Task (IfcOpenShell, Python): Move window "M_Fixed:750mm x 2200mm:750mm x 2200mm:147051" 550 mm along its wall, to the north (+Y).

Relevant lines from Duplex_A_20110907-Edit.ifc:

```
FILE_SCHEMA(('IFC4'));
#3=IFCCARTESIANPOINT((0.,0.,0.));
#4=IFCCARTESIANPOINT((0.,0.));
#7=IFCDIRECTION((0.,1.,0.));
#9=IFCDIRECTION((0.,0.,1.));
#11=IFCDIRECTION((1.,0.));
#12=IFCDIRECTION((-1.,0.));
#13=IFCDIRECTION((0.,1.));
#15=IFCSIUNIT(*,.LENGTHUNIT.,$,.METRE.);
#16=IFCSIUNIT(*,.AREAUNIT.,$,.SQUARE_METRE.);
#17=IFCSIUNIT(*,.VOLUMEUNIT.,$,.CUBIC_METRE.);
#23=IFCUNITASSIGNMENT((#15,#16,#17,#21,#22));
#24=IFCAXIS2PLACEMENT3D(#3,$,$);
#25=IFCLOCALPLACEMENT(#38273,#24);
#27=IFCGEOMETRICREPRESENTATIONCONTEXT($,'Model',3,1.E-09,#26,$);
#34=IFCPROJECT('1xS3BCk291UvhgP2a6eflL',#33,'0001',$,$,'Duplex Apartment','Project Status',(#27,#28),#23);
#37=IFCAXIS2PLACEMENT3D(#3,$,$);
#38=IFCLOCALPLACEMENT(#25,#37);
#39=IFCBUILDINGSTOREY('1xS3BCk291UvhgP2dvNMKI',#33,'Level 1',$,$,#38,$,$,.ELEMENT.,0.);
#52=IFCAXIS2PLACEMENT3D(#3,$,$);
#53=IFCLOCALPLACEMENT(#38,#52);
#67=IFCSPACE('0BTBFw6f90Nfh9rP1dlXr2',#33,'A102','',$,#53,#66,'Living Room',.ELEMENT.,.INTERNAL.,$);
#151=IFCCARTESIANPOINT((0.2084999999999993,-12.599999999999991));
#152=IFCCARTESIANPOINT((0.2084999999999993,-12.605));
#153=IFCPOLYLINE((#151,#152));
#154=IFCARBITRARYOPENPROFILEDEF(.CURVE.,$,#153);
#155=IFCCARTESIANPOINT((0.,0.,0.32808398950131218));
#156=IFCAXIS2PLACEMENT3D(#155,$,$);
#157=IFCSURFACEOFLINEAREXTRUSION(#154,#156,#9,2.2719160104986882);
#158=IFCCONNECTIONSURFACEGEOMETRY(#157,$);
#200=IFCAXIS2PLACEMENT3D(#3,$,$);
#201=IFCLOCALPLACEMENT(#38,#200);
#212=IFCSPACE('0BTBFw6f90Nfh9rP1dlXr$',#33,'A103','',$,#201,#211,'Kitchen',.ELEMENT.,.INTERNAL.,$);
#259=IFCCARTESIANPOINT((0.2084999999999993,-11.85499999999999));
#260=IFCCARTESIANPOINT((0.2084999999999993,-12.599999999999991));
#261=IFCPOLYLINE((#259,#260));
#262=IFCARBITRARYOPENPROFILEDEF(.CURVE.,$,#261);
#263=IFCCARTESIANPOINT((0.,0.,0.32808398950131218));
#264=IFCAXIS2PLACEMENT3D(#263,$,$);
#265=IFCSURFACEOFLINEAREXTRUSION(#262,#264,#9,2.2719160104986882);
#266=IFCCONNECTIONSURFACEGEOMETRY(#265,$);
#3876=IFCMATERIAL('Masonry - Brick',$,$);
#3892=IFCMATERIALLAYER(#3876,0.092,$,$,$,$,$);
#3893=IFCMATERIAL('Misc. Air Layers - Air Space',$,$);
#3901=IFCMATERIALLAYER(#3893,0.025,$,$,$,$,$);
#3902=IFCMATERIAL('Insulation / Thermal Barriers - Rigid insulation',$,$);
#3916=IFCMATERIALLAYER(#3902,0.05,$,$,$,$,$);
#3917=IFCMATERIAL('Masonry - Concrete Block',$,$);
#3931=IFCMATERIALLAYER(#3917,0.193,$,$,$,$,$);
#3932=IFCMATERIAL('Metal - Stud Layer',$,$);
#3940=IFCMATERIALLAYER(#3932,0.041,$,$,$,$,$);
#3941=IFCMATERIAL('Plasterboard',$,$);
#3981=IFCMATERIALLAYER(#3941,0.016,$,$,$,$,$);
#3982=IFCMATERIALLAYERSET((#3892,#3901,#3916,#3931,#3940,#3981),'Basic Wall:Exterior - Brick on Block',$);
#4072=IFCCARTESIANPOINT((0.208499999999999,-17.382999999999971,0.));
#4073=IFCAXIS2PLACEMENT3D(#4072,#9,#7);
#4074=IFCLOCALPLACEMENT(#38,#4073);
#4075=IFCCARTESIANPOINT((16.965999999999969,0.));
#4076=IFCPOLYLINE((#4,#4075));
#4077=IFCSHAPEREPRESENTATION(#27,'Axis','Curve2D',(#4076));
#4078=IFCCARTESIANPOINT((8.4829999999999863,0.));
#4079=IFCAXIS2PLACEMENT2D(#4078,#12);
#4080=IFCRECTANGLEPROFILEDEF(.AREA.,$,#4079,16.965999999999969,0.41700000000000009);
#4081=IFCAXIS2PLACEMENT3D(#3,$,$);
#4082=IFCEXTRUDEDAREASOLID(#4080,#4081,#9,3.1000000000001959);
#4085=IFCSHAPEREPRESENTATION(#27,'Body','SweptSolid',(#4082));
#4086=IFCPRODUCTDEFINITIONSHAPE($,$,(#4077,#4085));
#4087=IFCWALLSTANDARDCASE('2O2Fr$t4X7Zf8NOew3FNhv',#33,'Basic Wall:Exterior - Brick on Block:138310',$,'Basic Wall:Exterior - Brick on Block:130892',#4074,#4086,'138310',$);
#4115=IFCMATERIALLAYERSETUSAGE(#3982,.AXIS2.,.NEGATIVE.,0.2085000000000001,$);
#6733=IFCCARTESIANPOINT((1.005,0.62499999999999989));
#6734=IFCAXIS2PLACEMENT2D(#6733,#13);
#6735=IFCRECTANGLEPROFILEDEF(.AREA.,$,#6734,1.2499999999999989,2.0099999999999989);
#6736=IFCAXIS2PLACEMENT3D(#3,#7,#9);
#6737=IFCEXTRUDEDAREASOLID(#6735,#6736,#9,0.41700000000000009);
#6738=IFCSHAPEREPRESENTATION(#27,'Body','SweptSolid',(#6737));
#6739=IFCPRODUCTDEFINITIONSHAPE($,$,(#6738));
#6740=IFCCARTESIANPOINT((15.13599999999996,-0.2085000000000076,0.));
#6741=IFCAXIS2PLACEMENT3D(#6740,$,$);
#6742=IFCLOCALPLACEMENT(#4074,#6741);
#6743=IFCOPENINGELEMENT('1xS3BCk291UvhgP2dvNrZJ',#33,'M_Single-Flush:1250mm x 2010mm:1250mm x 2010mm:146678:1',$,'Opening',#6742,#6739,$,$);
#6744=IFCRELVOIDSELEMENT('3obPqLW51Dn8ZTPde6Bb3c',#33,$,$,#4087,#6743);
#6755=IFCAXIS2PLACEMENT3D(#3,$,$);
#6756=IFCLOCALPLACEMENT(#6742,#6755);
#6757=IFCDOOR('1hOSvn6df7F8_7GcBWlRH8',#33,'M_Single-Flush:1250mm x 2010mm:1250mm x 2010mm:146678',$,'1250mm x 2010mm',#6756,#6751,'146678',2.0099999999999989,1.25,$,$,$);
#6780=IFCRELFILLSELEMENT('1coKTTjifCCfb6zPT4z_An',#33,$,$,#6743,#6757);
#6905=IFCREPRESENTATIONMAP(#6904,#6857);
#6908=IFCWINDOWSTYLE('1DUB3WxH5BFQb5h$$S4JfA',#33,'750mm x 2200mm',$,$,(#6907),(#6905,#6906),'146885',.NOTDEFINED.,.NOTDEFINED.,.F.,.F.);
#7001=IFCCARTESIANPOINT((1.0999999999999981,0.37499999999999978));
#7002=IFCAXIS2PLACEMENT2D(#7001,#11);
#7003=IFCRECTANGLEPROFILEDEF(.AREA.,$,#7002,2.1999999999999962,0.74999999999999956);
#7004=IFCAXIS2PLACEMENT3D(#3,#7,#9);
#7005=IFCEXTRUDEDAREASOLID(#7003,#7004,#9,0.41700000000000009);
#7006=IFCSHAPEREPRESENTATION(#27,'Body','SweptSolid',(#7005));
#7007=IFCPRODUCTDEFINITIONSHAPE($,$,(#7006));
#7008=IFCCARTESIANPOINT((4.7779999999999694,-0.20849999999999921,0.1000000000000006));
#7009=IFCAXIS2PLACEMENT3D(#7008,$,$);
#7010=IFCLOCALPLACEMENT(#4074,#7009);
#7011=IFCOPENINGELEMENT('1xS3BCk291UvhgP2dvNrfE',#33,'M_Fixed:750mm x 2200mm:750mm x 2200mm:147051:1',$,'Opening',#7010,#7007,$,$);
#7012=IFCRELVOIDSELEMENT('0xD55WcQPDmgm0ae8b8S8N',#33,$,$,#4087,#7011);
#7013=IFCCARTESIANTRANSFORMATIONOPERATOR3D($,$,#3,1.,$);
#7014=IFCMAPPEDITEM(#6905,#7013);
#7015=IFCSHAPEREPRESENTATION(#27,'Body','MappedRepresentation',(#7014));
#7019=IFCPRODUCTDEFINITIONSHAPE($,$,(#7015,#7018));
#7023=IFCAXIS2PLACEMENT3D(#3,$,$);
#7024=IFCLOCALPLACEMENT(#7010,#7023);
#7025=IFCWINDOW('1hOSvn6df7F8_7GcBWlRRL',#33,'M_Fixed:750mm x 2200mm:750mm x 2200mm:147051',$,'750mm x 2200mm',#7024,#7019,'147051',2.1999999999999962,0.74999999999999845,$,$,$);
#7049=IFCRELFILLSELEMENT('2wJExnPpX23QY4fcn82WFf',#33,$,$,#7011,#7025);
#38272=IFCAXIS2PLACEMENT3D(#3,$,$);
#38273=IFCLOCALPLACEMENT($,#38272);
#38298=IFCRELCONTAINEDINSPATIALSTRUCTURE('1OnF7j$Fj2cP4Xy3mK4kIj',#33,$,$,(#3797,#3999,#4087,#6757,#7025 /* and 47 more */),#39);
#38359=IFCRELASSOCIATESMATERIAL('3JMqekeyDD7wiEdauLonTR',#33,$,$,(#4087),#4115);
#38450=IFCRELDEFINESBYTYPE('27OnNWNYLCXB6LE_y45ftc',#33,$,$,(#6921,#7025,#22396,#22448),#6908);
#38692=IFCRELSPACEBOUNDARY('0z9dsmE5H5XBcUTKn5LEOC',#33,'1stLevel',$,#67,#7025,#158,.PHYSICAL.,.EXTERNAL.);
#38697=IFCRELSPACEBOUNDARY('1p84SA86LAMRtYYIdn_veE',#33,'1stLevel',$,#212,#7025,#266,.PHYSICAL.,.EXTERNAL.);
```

```python
import numpy as np
import ifcopenshell
import ifcopenshell.api.geometry
import ifcopenshell.util.placement
import ifcopenshell.util.unit

model = ifcopenshell.open("Duplex_A_20110907-Edit.ifc")
unit_scale = ifcopenshell.util.unit.calculate_unit_scale(model)

window = model.by_guid("1hOSvn6df7F8_7GcBWlRRL")
opening = window.FillsVoids[0].RelatingOpeningElement
wall = opening.VoidsElements[0].RelatingBuildingElement

wall_matrix = ifcopenshell.util.placement.get_local_placement(wall.ObjectPlacement)
shift = wall_matrix[:3, 0] * 0.55 / unit_scale
before = ifcopenshell.util.placement.get_local_placement(window.ObjectPlacement)[:3, 3].copy()

# The window is placed relative to its opening, so it follows when the opening moves.
matrix = ifcopenshell.util.placement.get_local_placement(opening.ObjectPlacement)
matrix[:3, 3] += shift
ifcopenshell.api.geometry.edit_object_placement(
    model, product=opening, matrix=matrix, is_si=False, should_transform_children=True
)

# Space boundary surfaces are stored in each space's coordinates; move them too.
for rel in window.ProvidesBoundaries:
    if not rel.ConnectionGeometry:
        continue
    surface = rel.ConnectionGeometry.SurfaceOnRelatingElement
    space_matrix = ifcopenshell.util.placement.get_local_placement(rel.RelatingSpace.ObjectPlacement)
    point = np.array(surface.Position.Location.Coordinates) + space_matrix[:3, :3].T @ shift
    surface.Position = model.createIfcAxis2Placement3D(
        model.createIfcCartesianPoint(point.tolist()), surface.Position.Axis, surface.Position.RefDirection
    )

after = ifcopenshell.util.placement.get_local_placement(window.ObjectPlacement)[:3, 3]
print("window moved by", (after - before).round(3) + 0.0)

model.write("Duplex_A_20110907-Edit-out.ifc")
```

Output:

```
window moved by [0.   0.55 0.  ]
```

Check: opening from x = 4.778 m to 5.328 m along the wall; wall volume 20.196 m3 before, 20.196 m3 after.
